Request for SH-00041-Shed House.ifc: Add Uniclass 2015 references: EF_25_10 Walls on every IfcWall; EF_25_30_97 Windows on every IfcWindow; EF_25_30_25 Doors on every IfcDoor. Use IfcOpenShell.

First a look at what the model holds.

```python
import ifcopenshell

model = ifcopenshell.open("SH-00041-Shed House.ifc")
print(model.schema)
print("classifications:", [c.Name for c in model.by_type("IfcClassification")])
for ifc_class in ("IfcDoor", "IfcRoof", "IfcStair", "IfcWall", "IfcWindow"):
    print(ifc_class, len(model.by_type(ifc_class)))
```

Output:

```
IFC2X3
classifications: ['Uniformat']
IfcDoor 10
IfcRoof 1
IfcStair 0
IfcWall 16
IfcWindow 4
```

```python
import ifcopenshell
import ifcopenshell.api.classification

model = ifcopenshell.open("SH-00041-Shed House.ifc")

# IFC2X3 requires Source and Edition and has no link from the project to the system.
system = model.create_entity("IfcClassification", Source="NBS", Edition="2015", Name="Uniclass 2015")

codes = {
    "IfcWall": ("EF_25_10", "Walls"),
    "IfcWindow": ("EF_25_30_97", "Windows"),
    "IfcDoor": ("EF_25_30_25", "Doors"),
}
for ifc_class, (code, name) in codes.items():
    products = model.by_type(ifc_class)
    ifcopenshell.api.classification.add_reference(
        model, products=products, classification=system, identification=code, name=name
    )
    print(code, len(products))

model.write("SH-00041-Shed House_v2.ifc")
```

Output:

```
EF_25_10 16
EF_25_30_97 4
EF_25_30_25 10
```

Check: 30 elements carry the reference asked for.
